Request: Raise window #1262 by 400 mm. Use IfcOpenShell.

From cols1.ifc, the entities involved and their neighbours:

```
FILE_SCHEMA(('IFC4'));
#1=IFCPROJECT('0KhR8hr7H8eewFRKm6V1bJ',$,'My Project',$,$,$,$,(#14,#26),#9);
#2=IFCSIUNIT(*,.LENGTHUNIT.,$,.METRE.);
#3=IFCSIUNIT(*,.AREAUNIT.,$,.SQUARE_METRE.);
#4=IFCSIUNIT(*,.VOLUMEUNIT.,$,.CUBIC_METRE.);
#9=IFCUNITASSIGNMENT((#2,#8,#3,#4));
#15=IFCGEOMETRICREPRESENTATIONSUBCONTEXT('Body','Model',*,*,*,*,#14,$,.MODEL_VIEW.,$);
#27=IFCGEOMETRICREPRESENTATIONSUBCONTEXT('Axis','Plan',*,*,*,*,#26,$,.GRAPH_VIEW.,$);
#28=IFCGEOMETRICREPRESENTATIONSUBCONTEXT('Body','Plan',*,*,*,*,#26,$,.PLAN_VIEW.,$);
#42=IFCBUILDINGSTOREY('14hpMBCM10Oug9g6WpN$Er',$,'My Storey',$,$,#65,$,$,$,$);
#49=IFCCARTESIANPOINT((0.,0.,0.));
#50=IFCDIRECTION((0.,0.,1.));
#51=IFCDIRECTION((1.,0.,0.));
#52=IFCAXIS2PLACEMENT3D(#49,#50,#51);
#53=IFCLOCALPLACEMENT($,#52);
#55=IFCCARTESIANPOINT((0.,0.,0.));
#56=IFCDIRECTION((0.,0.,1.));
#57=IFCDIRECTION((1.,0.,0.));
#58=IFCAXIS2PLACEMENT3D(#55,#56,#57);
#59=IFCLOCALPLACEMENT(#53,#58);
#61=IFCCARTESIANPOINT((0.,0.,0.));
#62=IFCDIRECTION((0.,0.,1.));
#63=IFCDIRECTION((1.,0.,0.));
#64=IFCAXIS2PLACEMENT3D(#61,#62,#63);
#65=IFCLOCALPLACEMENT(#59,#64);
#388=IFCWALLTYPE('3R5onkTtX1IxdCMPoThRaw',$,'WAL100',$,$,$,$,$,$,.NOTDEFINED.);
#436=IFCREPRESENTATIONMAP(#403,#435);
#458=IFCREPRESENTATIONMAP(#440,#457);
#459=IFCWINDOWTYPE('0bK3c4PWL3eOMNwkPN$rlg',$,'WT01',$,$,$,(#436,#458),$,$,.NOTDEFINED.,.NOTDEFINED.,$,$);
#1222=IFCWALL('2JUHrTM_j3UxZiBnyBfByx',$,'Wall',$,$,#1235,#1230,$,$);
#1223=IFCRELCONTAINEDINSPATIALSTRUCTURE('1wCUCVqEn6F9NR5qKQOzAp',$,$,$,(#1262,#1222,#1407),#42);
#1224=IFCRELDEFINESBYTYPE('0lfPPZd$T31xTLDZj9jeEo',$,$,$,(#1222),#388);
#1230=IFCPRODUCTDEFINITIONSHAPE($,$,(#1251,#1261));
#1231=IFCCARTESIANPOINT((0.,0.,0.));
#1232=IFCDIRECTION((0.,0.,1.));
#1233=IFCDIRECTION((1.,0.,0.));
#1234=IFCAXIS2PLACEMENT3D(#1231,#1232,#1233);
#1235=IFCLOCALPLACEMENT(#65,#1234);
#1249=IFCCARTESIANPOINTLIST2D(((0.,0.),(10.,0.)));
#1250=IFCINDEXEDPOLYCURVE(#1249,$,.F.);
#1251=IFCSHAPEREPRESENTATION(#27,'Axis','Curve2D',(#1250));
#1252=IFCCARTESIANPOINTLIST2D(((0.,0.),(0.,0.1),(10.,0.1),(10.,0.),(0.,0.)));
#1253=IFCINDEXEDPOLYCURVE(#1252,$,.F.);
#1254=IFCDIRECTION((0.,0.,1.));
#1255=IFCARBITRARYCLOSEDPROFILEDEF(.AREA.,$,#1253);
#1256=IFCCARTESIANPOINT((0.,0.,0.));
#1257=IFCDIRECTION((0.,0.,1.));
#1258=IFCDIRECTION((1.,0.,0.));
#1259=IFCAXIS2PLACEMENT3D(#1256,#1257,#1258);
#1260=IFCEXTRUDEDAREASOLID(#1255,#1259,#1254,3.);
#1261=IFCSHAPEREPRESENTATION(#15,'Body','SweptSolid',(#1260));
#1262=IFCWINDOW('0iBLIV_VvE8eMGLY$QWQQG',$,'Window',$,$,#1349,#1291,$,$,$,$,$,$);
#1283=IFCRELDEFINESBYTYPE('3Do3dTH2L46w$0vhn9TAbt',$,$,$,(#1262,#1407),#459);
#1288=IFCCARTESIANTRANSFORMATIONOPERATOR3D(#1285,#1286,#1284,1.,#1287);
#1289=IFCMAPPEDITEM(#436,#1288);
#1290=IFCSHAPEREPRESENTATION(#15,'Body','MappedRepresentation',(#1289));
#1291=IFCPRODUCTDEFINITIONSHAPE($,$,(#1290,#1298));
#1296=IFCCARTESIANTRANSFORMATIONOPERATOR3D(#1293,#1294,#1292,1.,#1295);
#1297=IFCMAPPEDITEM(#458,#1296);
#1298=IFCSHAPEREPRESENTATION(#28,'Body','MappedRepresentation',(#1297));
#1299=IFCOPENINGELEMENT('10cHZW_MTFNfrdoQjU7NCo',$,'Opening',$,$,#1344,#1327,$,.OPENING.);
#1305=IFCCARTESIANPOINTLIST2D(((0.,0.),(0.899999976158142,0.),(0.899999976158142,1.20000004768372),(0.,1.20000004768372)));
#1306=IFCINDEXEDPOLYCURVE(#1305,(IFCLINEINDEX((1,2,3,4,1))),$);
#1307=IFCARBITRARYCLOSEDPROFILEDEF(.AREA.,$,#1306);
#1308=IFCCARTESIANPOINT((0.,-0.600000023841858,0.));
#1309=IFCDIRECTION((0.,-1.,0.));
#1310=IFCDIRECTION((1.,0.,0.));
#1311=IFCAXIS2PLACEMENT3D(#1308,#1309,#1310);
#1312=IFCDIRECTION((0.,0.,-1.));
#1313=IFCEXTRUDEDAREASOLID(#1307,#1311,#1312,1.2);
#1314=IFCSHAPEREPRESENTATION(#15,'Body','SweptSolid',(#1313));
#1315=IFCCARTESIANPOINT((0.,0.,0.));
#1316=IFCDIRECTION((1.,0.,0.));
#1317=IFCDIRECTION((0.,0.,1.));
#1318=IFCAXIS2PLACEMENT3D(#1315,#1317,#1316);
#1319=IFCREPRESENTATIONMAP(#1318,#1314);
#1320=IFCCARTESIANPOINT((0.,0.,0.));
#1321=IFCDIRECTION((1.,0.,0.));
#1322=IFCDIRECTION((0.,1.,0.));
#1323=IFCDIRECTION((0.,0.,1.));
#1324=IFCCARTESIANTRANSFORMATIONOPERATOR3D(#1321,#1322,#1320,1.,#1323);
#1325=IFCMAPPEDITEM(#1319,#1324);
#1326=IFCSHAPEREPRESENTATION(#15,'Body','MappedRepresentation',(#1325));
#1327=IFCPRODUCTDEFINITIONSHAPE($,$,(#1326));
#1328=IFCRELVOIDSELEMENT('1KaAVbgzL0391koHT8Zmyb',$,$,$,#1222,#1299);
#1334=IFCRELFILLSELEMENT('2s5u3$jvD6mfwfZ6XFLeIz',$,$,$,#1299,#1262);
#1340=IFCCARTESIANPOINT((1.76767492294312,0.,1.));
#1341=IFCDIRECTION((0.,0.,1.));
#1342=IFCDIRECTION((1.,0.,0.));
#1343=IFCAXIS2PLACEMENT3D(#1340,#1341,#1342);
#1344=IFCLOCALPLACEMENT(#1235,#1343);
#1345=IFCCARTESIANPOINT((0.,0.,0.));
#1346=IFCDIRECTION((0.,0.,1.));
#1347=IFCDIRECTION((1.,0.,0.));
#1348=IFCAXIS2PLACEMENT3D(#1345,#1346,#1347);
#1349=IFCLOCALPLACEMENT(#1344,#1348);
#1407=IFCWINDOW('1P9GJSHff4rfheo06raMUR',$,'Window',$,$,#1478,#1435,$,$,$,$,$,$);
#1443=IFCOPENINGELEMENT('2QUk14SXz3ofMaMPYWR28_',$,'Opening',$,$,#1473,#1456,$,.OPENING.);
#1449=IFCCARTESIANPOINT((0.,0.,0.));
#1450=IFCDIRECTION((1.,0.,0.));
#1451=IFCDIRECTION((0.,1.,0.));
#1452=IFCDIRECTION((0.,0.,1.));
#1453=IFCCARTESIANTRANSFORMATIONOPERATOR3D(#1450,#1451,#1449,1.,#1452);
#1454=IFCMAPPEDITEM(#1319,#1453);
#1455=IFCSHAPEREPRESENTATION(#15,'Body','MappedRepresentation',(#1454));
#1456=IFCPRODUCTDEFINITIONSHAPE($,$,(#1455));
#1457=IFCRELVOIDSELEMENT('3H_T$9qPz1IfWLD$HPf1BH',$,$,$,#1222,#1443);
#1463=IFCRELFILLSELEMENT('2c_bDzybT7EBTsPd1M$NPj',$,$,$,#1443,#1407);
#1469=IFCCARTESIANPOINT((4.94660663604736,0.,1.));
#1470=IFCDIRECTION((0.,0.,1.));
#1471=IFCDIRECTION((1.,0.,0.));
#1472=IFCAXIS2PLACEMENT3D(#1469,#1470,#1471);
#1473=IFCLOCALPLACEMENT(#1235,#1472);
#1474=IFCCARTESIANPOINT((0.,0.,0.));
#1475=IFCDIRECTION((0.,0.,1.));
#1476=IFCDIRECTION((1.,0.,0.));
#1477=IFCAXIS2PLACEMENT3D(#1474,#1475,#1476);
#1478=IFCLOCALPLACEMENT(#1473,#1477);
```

```python
import numpy as np
import ifcopenshell
import ifcopenshell.api.geometry
import ifcopenshell.util.placement
import ifcopenshell.util.unit

model = ifcopenshell.open("cols1.ifc")
unit_scale = ifcopenshell.util.unit.calculate_unit_scale(model)

window = model.by_guid("0iBLIV_VvE8eMGLY$QWQQG")
opening = window.FillsVoids[0].RelatingOpeningElement
dz = 0.4

shift = np.array([0.0, 0.0, dz])
# The window is placed relative to its opening, so it follows when the opening moves.
matrix = ifcopenshell.util.placement.get_local_placement(opening.ObjectPlacement)
matrix[:3, 3] += shift
ifcopenshell.api.geometry.edit_object_placement(
    model, product=opening, matrix=matrix, is_si=False, should_transform_children=True
)

print(f"moved by {dz * unit_scale:+.3f} m")

model.write("cols1_v2.ifc")
```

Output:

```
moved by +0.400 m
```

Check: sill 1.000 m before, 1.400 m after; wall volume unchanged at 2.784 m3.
